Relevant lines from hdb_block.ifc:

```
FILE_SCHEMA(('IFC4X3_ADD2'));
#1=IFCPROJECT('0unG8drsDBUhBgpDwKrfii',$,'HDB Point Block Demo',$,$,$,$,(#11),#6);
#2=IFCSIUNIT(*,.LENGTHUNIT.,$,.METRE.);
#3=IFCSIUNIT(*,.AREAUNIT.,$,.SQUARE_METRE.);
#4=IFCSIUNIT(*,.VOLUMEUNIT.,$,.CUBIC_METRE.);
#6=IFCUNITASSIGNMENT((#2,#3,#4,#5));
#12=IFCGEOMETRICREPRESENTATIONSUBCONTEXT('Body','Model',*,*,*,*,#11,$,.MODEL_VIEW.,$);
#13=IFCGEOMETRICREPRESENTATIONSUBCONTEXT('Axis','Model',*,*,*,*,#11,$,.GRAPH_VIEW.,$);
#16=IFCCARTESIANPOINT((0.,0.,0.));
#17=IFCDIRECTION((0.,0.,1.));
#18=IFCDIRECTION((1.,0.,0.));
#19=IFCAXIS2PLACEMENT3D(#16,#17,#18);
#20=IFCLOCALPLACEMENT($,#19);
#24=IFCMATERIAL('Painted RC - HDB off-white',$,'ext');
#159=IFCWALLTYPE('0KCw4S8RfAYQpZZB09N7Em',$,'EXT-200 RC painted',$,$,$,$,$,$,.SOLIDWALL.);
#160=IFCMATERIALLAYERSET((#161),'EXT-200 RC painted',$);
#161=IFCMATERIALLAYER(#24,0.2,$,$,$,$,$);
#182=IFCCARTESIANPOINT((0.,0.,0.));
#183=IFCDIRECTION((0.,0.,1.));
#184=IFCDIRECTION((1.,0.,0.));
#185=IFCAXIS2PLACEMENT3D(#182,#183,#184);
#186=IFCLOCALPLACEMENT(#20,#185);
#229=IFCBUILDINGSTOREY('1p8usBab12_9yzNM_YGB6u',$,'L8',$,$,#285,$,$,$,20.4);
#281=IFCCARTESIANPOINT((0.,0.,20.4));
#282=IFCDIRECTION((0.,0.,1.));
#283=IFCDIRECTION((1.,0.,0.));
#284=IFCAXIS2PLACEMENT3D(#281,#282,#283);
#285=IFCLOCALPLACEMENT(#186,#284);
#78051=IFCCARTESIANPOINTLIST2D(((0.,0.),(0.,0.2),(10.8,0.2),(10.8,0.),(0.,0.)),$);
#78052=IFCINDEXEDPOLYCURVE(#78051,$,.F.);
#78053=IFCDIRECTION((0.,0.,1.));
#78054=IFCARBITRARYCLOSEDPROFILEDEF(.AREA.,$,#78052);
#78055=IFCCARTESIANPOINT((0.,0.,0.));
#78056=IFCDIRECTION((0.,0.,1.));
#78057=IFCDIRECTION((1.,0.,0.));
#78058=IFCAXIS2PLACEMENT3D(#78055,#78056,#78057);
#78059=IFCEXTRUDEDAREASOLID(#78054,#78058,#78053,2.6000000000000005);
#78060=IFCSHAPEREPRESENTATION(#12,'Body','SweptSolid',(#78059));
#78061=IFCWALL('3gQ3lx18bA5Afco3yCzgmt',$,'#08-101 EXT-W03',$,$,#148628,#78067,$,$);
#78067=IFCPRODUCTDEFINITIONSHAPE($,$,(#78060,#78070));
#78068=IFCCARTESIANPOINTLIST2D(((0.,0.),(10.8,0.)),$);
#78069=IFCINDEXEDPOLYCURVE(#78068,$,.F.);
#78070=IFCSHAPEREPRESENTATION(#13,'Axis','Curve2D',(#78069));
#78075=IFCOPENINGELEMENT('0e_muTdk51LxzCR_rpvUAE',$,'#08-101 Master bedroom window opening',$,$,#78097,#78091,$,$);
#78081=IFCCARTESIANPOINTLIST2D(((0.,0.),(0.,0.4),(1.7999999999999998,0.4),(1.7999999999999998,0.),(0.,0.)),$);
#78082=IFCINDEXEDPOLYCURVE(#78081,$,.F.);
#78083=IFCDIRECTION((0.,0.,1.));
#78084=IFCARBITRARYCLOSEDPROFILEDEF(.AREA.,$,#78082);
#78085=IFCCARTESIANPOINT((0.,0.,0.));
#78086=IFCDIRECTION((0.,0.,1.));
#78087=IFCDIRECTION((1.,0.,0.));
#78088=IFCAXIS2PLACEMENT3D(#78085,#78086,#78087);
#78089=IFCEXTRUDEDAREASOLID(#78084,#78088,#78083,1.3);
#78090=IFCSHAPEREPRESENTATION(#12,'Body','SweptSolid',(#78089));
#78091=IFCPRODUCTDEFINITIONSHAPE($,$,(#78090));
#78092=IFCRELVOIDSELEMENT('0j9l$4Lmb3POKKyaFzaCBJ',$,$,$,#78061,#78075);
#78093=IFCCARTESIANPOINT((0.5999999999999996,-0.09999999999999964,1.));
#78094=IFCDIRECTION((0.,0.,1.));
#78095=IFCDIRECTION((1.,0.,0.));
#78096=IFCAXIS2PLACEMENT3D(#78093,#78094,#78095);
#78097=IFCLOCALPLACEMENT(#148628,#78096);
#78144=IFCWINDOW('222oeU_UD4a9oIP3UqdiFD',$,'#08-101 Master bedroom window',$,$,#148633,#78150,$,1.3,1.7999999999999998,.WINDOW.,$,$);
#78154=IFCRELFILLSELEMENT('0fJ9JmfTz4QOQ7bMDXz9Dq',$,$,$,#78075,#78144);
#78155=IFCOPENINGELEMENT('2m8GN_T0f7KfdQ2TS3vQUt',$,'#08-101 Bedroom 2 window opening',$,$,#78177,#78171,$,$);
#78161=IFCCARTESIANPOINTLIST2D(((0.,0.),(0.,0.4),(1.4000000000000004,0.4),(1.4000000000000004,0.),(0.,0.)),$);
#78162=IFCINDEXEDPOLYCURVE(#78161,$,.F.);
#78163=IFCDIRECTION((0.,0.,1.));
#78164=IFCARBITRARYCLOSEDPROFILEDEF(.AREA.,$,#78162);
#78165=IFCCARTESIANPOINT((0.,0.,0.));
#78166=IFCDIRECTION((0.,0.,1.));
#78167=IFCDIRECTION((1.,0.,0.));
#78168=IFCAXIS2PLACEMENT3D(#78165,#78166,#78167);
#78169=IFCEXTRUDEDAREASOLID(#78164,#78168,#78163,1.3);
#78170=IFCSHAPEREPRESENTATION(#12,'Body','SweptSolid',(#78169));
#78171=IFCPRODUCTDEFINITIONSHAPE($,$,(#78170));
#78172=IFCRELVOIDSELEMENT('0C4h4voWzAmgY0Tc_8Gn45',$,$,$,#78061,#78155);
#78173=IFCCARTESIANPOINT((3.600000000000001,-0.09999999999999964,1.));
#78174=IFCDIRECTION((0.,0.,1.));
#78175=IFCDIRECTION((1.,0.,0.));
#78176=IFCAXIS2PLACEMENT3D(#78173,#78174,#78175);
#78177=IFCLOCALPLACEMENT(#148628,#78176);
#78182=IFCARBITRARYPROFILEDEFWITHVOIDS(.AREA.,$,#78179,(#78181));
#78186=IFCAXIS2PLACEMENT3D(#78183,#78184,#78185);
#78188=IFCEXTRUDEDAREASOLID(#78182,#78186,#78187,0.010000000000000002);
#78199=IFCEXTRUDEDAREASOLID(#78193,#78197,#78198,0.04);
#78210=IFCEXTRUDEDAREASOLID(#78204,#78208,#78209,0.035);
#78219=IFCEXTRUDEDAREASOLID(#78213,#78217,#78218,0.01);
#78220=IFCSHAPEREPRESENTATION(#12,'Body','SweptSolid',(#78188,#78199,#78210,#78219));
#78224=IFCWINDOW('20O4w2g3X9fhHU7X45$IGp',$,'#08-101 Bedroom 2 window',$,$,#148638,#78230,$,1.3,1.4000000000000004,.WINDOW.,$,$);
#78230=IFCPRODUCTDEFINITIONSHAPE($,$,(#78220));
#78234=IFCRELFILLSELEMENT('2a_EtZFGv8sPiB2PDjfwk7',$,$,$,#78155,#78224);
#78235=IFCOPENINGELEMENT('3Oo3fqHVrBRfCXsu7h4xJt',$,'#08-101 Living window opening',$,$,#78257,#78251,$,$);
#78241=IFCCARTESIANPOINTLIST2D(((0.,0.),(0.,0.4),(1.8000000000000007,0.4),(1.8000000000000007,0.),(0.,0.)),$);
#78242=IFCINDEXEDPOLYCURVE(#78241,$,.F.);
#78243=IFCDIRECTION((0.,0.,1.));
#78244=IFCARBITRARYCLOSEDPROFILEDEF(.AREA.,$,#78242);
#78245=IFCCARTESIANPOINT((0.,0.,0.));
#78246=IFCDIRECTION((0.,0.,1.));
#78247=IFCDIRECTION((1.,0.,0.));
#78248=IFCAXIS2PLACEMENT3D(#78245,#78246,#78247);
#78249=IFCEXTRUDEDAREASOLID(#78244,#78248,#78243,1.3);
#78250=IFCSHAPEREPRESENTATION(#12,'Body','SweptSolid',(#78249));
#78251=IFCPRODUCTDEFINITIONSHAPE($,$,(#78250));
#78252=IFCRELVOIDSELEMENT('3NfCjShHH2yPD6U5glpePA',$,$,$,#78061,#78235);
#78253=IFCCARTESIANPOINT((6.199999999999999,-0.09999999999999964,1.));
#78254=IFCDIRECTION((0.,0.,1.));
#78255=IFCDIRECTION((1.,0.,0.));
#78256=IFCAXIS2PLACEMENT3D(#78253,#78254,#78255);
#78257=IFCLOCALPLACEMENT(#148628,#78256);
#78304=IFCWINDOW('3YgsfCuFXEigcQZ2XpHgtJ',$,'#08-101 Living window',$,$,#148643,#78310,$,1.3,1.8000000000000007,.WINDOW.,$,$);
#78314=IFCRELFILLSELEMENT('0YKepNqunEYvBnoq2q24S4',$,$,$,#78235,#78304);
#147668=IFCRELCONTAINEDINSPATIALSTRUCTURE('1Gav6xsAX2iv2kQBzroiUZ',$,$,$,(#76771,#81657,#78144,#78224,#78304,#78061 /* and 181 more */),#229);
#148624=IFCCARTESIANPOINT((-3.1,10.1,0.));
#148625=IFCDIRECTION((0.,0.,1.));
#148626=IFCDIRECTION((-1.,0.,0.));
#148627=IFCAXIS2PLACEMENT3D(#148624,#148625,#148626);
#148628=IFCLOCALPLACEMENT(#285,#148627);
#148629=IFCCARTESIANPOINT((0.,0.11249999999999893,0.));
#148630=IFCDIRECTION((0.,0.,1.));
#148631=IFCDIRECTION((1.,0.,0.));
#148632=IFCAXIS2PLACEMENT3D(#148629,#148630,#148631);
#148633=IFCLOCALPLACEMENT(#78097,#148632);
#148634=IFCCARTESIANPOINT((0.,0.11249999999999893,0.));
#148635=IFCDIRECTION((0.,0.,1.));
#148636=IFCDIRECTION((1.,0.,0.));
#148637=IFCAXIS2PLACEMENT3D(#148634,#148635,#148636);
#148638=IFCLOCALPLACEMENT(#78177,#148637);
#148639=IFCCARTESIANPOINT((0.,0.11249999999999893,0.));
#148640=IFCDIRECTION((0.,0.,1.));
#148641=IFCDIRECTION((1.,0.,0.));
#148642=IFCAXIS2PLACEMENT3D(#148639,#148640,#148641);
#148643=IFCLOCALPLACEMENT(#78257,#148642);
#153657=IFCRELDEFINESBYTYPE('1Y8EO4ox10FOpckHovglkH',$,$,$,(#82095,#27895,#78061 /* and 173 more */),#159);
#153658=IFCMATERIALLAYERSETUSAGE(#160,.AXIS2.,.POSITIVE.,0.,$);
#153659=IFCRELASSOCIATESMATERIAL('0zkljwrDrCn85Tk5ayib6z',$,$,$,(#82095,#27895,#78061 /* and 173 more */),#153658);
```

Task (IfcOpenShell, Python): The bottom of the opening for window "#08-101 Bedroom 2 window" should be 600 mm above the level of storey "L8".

```python
import numpy as np
import ifcopenshell
import ifcopenshell.api.geometry
import ifcopenshell.geom
import ifcopenshell.util.element
import ifcopenshell.util.placement
import ifcopenshell.util.shape
import ifcopenshell.util.unit

model = ifcopenshell.open("hdb_block.ifc")
unit_scale = ifcopenshell.util.unit.calculate_unit_scale(model)

window = model.by_id(78224)
opening = window.FillsVoids[0].RelatingOpeningElement
storey = ifcopenshell.util.element.get_container(window, ifc_class="IfcBuildingStorey")
level = ifcopenshell.util.placement.get_local_placement(storey.ObjectPlacement)[2, 3]

# The opening's origin need not be at the sill, so measure its lowest point.
shape = ifcopenshell.geom.create_shape(ifcopenshell.geom.settings(), opening)
bottom = ifcopenshell.util.shape.get_shape_bottom_elevation(shape, shape.geometry) / unit_scale
dz = level + 0.6 / unit_scale - bottom

shift = np.array([0.0, 0.0, dz])
# The window is placed relative to its opening, so it follows when the opening moves.
matrix = ifcopenshell.util.placement.get_local_placement(opening.ObjectPlacement)
matrix[:3, 3] += shift
ifcopenshell.api.geometry.edit_object_placement(
    model, product=opening, matrix=matrix, is_si=False, should_transform_children=True
)

print(f"moved by {dz * unit_scale:+.3f} m")

model.write("hdb_block-out.ifc")
```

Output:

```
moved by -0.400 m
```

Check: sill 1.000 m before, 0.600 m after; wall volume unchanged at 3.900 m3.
